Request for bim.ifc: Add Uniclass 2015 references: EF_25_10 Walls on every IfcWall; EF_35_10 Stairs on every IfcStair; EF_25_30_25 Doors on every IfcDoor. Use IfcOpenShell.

First a look at what the model holds.

```python
import ifcopenshell

model = ifcopenshell.open("bim.ifc")
print(model.schema)
print("classifications:", [c.Name for c in model.by_type("IfcClassification")])
for ifc_class in ("IfcDoor", "IfcRoof", "IfcStair", "IfcWall", "IfcWindow"):
    print(ifc_class, len(model.by_type(ifc_class)))
```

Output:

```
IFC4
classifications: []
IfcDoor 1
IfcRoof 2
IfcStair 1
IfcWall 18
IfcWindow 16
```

```python
import ifcopenshell
import ifcopenshell.api.classification

model = ifcopenshell.open("bim.ifc")

system = ifcopenshell.api.classification.add_classification(model, classification="Uniclass 2015")

codes = {
    "IfcWall": ("EF_25_10", "Walls"),
    "IfcStair": ("EF_35_10", "Stairs"),
    "IfcDoor": ("EF_25_30_25", "Doors"),
}
for ifc_class, (code, name) in codes.items():
    products = model.by_type(ifc_class)
    ifcopenshell.api.classification.add_reference(
        model, products=products, classification=system, identification=code, name=name
    )
    print(code, len(products))

model.write("bim-out.ifc")
```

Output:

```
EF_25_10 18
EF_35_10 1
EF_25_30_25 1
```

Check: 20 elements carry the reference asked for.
